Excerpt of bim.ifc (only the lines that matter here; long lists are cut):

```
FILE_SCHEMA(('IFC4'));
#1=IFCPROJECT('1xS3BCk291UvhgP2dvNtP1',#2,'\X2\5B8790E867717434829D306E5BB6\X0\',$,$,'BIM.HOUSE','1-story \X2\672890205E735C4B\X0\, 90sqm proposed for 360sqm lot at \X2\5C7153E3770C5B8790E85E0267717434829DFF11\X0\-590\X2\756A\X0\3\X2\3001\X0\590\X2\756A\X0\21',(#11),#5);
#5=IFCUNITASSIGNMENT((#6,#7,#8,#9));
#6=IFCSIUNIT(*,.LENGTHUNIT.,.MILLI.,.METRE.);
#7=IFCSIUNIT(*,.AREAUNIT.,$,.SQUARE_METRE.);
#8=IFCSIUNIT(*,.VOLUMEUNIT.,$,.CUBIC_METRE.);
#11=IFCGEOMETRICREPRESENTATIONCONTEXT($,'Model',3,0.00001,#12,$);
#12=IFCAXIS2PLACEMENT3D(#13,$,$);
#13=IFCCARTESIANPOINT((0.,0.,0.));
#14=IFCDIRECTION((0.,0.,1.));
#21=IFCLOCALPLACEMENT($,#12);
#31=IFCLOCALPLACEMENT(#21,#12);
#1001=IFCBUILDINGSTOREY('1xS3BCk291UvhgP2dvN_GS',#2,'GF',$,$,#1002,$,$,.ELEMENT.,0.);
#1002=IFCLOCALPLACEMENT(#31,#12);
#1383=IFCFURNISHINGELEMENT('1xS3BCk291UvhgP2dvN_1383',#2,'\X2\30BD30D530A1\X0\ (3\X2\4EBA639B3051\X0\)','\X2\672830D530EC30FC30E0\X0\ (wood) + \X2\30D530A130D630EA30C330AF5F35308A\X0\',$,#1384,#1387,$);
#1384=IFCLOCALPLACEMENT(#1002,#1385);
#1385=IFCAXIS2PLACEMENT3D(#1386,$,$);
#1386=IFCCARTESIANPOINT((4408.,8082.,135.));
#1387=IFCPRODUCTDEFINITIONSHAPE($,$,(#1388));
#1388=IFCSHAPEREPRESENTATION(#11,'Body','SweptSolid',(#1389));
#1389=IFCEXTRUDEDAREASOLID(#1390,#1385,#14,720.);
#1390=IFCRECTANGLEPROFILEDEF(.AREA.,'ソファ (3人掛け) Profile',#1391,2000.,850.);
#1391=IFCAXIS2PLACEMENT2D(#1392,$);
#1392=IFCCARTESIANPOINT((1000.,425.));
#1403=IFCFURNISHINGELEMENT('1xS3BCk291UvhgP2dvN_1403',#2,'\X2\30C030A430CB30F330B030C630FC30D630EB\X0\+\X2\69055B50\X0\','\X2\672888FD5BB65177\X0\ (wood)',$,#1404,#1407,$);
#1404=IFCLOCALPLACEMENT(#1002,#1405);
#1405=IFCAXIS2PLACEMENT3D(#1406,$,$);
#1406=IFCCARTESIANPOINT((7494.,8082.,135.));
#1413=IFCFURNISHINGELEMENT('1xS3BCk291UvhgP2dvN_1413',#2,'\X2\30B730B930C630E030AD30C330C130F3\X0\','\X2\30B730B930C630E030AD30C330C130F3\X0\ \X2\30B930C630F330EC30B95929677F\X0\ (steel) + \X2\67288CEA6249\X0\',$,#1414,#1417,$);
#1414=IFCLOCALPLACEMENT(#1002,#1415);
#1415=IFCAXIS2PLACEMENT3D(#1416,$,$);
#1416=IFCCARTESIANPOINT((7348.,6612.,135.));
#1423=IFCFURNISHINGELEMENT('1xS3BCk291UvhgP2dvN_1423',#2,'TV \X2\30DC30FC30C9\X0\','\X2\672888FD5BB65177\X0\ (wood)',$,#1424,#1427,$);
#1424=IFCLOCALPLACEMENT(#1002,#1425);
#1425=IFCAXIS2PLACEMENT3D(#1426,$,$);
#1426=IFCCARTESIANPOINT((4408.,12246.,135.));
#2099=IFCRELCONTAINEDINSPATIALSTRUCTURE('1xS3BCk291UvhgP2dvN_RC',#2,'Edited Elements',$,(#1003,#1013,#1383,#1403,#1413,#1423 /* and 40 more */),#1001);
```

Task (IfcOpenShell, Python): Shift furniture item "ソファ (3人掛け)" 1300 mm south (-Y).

```python
import ifcopenshell
import ifcopenshell.api.geometry
import ifcopenshell.util.placement

model = ifcopenshell.open("bim.ifc")

item = model.by_guid("1xS3BCk291UvhgP2dvN_1383")
matrix = ifcopenshell.util.placement.get_local_placement(item.ObjectPlacement)
matrix[1, 3] -= 1300.0
ifcopenshell.api.geometry.edit_object_placement(model, product=item, matrix=matrix, is_si=False)

print(ifcopenshell.util.placement.get_local_placement(item.ObjectPlacement).round(3) + 0.0)

model.write("bim_rev.ifc")
```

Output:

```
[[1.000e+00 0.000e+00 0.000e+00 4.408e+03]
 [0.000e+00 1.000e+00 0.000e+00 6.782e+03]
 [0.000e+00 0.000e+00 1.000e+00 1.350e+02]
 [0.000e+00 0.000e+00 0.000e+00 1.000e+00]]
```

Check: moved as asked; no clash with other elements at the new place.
